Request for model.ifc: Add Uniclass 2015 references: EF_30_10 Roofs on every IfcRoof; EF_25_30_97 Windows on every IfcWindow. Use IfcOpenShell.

First a look at what the model holds.

```python
import ifcopenshell

model = ifcopenshell.open("model.ifc")
print(model.schema)
print("classifications:", [c.Name for c in model.by_type("IfcClassification")])
for ifc_class in ("IfcDoor", "IfcRoof", "IfcStair", "IfcWall", "IfcWindow"):
    print(ifc_class, len(model.by_type(ifc_class)))
```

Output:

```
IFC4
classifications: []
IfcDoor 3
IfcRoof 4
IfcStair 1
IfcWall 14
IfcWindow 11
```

```python
import ifcopenshell
import ifcopenshell.api.classification

model = ifcopenshell.open("model.ifc")

system = ifcopenshell.api.classification.add_classification(model, classification="Uniclass 2015")

codes = {
    "IfcRoof": ("EF_30_10", "Roofs"),
    "IfcWindow": ("EF_25_30_97", "Windows"),
}
for ifc_class, (code, name) in codes.items():
    products = model.by_type(ifc_class)
    ifcopenshell.api.classification.add_reference(
        model, products=products, classification=system, identification=code, name=name
    )
    print(code, len(products))

model.write("model_v2.ifc")
```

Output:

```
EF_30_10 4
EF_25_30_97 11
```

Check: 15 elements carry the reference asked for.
